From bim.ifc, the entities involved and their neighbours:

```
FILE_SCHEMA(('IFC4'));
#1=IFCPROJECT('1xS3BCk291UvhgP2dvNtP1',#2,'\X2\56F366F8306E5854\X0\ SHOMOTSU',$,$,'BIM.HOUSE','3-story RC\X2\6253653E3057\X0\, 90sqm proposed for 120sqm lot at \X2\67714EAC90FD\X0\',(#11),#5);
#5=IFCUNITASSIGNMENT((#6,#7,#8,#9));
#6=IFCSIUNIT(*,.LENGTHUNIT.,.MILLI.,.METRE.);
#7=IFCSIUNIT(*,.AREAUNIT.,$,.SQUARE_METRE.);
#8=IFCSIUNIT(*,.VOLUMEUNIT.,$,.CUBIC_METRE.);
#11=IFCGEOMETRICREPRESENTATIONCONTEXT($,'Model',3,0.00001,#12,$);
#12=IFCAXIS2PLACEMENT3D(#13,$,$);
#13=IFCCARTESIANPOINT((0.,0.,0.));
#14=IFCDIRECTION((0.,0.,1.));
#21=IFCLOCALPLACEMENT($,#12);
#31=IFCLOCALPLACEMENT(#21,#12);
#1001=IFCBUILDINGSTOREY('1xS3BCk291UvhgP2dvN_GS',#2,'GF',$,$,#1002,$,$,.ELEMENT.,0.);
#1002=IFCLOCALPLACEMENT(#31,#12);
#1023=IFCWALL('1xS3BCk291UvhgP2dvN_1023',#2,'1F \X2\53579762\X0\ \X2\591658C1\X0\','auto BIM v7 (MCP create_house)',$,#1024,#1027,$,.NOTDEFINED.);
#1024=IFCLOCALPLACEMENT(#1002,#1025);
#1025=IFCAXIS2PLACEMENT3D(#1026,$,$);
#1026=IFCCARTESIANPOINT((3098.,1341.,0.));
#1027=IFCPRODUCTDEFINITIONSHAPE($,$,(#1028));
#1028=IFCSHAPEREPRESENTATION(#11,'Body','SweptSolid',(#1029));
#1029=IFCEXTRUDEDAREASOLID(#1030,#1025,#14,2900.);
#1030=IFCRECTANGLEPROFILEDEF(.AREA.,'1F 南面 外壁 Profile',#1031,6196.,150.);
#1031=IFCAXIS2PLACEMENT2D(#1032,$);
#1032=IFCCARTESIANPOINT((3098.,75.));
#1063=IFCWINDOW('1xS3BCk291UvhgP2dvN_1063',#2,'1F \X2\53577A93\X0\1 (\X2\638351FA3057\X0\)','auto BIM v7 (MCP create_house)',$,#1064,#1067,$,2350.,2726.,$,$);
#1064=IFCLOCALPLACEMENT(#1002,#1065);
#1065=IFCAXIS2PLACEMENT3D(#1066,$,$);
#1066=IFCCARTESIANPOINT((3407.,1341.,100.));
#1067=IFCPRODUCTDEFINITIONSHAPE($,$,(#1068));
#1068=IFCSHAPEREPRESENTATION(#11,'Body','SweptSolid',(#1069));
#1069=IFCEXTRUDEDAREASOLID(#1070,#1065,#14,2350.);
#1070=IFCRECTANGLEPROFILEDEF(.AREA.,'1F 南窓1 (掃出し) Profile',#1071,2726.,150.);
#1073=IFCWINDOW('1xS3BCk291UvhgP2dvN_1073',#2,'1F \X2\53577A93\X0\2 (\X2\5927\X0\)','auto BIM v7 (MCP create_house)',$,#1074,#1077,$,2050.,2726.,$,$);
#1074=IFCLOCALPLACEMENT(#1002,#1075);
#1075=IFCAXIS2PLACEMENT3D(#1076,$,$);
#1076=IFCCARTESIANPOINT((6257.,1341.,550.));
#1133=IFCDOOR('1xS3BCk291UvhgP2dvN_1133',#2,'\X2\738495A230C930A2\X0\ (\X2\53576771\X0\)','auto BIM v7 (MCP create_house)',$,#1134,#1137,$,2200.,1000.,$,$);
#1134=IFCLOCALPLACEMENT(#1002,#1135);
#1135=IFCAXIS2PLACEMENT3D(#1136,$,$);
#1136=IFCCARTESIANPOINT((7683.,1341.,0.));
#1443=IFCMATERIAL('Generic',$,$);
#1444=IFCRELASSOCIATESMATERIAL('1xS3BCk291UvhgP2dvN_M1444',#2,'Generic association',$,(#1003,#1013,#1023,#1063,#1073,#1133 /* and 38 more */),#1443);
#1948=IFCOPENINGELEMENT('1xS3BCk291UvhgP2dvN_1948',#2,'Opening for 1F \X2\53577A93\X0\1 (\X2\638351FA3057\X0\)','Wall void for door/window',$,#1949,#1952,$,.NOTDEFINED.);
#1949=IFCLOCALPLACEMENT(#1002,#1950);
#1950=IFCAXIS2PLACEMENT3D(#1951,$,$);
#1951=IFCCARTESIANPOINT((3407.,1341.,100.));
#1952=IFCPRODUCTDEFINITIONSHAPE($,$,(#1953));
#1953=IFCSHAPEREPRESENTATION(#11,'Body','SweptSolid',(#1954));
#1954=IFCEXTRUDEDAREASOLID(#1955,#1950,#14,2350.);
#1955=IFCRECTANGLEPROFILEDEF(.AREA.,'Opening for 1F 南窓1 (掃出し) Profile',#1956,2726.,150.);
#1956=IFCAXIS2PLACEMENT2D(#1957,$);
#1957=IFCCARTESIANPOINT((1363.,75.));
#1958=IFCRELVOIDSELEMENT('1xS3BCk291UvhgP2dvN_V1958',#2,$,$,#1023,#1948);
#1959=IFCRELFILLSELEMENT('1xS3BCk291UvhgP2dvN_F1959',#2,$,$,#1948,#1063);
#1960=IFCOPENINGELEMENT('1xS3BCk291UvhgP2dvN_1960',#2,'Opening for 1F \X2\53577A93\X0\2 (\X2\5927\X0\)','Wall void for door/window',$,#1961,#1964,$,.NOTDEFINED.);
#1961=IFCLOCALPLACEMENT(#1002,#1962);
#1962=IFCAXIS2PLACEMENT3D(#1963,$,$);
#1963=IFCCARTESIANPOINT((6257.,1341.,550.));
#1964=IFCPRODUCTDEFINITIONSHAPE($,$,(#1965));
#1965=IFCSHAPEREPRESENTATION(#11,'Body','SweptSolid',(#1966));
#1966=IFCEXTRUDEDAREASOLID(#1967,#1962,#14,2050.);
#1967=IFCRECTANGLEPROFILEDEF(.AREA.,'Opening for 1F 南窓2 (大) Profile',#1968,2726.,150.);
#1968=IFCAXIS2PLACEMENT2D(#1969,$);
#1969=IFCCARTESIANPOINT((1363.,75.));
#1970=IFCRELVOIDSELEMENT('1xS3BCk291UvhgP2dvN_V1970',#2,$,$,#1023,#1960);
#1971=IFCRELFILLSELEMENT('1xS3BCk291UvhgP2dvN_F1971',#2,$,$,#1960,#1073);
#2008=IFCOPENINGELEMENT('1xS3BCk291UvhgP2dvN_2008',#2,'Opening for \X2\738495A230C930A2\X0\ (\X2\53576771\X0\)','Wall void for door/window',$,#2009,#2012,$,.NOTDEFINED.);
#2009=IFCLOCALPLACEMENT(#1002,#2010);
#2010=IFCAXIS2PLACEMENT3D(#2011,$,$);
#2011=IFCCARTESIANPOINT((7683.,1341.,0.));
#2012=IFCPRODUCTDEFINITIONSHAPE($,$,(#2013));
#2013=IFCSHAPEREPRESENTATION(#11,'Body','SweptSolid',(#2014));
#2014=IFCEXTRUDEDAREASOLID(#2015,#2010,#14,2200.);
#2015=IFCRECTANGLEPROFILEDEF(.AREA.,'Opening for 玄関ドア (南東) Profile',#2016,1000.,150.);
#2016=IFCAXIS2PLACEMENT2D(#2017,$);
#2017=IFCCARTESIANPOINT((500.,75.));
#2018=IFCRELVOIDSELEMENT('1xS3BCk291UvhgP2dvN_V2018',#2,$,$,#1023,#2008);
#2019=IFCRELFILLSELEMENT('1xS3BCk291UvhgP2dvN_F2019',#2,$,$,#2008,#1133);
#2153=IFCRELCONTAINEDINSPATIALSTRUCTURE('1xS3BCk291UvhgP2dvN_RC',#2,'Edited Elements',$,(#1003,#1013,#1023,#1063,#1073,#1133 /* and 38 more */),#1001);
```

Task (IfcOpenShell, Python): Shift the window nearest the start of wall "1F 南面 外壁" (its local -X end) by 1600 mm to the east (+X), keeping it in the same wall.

```python
import ifcopenshell
import ifcopenshell.api.geometry
import ifcopenshell.util.placement
import ifcopenshell.util.unit

model = ifcopenshell.open("bim.ifc")
unit_scale = ifcopenshell.util.unit.calculate_unit_scale(model)

window = model.by_guid("1xS3BCk291UvhgP2dvN_1063")
opening = window.FillsVoids[0].RelatingOpeningElement
wall = opening.VoidsElements[0].RelatingBuildingElement

wall_matrix = ifcopenshell.util.placement.get_local_placement(wall.ObjectPlacement)
shift = wall_matrix[:3, 0] * 1.6 / unit_scale
before = ifcopenshell.util.placement.get_local_placement(window.ObjectPlacement)[:3, 3].copy()

# The window is not placed relative to its opening, so move both.
for product in (opening, window):
    matrix = ifcopenshell.util.placement.get_local_placement(product.ObjectPlacement)
    matrix[:3, 3] += shift
    ifcopenshell.api.geometry.edit_object_placement(model, product=product, matrix=matrix, is_si=False)

after = ifcopenshell.util.placement.get_local_placement(window.ObjectPlacement)[:3, 3]
print("window moved by", (after - before).round(3) + 0.0)

model.write("bim_edited.ifc")
```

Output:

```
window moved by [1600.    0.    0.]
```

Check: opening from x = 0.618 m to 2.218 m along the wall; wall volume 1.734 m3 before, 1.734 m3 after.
